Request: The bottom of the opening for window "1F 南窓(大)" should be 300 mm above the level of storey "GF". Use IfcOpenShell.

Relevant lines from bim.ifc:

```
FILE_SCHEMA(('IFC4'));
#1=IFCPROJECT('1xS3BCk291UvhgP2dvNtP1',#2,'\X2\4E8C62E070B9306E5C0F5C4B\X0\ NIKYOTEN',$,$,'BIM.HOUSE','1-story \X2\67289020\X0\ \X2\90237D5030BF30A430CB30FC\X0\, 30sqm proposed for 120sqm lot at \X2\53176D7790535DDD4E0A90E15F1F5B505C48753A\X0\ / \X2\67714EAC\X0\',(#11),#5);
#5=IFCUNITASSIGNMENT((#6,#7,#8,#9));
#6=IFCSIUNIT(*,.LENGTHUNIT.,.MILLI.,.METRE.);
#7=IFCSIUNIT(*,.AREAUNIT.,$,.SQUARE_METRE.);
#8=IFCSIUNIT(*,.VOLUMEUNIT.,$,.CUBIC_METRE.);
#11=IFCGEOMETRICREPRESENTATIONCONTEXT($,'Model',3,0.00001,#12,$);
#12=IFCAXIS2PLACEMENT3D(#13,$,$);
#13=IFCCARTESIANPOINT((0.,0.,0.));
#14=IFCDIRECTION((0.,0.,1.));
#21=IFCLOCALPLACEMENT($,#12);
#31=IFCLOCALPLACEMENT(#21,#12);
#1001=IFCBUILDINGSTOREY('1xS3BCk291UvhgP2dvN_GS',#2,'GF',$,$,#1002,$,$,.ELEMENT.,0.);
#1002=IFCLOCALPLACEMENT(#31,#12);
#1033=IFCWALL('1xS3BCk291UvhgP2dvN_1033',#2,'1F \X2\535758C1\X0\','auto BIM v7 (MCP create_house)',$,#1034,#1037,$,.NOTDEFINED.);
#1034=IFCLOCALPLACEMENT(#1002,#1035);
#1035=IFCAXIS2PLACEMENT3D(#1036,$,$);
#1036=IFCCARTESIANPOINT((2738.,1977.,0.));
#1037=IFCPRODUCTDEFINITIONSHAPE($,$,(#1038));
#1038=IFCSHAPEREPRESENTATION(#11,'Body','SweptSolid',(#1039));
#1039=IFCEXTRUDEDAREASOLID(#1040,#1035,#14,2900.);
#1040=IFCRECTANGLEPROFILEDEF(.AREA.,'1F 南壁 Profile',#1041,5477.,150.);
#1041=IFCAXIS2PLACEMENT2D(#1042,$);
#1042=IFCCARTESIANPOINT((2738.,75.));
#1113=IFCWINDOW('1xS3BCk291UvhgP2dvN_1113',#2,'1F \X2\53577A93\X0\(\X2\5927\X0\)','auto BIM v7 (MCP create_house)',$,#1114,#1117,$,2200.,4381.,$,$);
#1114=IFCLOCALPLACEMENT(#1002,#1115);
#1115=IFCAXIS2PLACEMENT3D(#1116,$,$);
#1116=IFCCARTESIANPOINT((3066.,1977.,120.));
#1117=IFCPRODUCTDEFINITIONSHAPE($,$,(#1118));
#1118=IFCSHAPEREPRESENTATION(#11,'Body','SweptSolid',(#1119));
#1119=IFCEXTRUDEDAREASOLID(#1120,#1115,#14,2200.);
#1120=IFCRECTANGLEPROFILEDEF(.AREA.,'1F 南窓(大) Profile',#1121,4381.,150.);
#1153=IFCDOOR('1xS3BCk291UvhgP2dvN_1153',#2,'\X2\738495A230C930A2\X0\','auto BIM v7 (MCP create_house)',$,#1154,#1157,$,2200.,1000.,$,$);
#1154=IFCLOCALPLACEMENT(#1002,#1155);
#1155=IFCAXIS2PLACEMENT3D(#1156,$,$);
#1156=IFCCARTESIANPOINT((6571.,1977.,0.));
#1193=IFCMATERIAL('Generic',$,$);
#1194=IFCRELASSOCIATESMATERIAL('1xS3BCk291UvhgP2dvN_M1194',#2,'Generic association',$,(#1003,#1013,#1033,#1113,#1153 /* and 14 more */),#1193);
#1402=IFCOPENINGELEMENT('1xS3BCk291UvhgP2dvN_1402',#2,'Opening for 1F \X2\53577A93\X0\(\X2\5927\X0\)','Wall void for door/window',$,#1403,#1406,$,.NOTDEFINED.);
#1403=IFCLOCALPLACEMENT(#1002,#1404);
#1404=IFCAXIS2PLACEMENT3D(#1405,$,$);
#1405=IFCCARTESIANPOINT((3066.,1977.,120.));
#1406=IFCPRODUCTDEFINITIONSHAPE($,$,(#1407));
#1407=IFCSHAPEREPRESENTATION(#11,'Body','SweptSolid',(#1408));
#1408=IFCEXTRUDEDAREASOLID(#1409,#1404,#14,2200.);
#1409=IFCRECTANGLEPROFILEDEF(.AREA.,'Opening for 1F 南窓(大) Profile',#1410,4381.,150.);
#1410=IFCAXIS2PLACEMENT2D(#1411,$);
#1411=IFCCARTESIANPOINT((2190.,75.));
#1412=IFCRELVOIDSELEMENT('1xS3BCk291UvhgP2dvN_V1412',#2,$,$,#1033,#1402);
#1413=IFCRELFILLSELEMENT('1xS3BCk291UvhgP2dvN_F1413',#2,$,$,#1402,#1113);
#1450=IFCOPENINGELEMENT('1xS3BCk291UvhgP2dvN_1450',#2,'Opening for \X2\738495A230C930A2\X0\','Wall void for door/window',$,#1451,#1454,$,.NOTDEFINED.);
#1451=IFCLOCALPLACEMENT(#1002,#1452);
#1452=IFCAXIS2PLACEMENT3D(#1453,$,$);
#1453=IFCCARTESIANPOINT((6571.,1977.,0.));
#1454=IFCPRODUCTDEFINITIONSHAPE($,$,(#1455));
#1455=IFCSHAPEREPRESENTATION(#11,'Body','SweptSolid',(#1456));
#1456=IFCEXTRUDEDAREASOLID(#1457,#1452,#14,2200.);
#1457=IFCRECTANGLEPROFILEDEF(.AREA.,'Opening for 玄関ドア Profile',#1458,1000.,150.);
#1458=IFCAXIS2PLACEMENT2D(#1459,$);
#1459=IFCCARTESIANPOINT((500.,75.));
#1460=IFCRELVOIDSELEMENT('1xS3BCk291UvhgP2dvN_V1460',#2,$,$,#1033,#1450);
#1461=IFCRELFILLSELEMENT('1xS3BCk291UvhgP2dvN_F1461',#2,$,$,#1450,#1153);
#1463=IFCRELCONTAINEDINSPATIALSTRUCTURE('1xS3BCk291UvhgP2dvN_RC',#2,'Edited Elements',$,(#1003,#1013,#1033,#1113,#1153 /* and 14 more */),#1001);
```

```python
import numpy as np
import ifcopenshell
import ifcopenshell.api.geometry
import ifcopenshell.geom
import ifcopenshell.util.element
import ifcopenshell.util.placement
import ifcopenshell.util.shape
import ifcopenshell.util.unit

model = ifcopenshell.open("bim.ifc")
unit_scale = ifcopenshell.util.unit.calculate_unit_scale(model)

window = model.by_guid("1xS3BCk291UvhgP2dvN_1113")
opening = window.FillsVoids[0].RelatingOpeningElement
storey = ifcopenshell.util.element.get_container(window, ifc_class="IfcBuildingStorey")
level = ifcopenshell.util.placement.get_local_placement(storey.ObjectPlacement)[2, 3]

# The opening's origin need not be at the sill, so measure its lowest point.
shape = ifcopenshell.geom.create_shape(ifcopenshell.geom.settings(), opening)
bottom = ifcopenshell.util.shape.get_shape_bottom_elevation(shape, shape.geometry) / unit_scale
dz = level + 0.3 / unit_scale - bottom

shift = np.array([0.0, 0.0, dz])
# The window is not placed relative to its opening, so move both.
for product in (opening, window):
    matrix = ifcopenshell.util.placement.get_local_placement(product.ObjectPlacement)
    matrix[:3, 3] += shift
    ifcopenshell.api.geometry.edit_object_placement(model, product=product, matrix=matrix, is_si=False)

print(f"moved by {dz * unit_scale:+.3f} m")

model.write("bim_rev.ifc")
```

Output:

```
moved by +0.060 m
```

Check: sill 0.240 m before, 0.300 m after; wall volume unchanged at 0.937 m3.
